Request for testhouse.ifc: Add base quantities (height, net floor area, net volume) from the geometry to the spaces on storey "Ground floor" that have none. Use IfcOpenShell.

First a look at what the model holds.

```python
import ifcopenshell
import ifcopenshell.util.element
import ifcopenshell.util.unit

model = ifcopenshell.open("testhouse.ifc")
print(model.schema)
for unit_type in ("LENGTHUNIT", "AREAUNIT", "VOLUMEUNIT"):
    print(unit_type, ifcopenshell.util.unit.calculate_unit_scale(model, unit_type))
storey = next(s for s in model.by_type("IfcBuildingStorey") if s.Name == "Ground floor")
spaces = [e for e in ifcopenshell.util.element.get_decomposition(storey) if e.is_a("IfcSpace")]
for e in sorted(spaces, key=lambda e: e.id()):
    print(e.id(), e.is_a(), e.Name, list(ifcopenshell.util.element.get_psets(e, qtos_only=True)), sep=" | ")
```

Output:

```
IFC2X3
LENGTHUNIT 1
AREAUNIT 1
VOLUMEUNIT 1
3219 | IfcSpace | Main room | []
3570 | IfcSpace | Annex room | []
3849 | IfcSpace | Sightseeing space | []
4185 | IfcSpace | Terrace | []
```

```python
import ifcopenshell
import ifcopenshell.api.pset
import ifcopenshell.geom
import ifcopenshell.util.element
import ifcopenshell.util.shape
import ifcopenshell.util.unit

model = ifcopenshell.open("testhouse.ifc")
unit_scale = ifcopenshell.util.unit.calculate_unit_scale(model)
area_scale = ifcopenshell.util.unit.calculate_unit_scale(model, "AREAUNIT")
volume_scale = ifcopenshell.util.unit.calculate_unit_scale(model, "VOLUMEUNIT")
settings = ifcopenshell.geom.settings()

storey = next(s for s in model.by_type("IfcBuildingStorey") if s.Name == "Ground floor")
spaces = [e for e in ifcopenshell.util.element.get_decomposition(storey) if e.is_a("IfcSpace")]

for e in sorted(spaces, key=lambda e: e.id()):
    if ifcopenshell.util.element.get_psets(e, qtos_only=True, should_inherit=False):
        continue
    # Geometry comes back in metres, in the element's own axes.
    shape = ifcopenshell.geom.create_shape(settings, e)
    values = {
        "Height": ifcopenshell.util.shape.get_z(shape.geometry) / unit_scale,
        "NetFloorArea": ifcopenshell.util.shape.get_footprint_area(shape.geometry) / area_scale,
        "NetVolume": ifcopenshell.util.shape.get_volume(shape.geometry) / volume_scale,
    }
    qto = ifcopenshell.api.pset.add_qto(model, product=e, name="BaseQuantities")
    ifcopenshell.api.pset.edit_qto(model, qto=qto, properties=values)
    print(e.id(), {k: round(v, 3) for k, v in values.items()})

model.write("testhouse-out.ifc")
```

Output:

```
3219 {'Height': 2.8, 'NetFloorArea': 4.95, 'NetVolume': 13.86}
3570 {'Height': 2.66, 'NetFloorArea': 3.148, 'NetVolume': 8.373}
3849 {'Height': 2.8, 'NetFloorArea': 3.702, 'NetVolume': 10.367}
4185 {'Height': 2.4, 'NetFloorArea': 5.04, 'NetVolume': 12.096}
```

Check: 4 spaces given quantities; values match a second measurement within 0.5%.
